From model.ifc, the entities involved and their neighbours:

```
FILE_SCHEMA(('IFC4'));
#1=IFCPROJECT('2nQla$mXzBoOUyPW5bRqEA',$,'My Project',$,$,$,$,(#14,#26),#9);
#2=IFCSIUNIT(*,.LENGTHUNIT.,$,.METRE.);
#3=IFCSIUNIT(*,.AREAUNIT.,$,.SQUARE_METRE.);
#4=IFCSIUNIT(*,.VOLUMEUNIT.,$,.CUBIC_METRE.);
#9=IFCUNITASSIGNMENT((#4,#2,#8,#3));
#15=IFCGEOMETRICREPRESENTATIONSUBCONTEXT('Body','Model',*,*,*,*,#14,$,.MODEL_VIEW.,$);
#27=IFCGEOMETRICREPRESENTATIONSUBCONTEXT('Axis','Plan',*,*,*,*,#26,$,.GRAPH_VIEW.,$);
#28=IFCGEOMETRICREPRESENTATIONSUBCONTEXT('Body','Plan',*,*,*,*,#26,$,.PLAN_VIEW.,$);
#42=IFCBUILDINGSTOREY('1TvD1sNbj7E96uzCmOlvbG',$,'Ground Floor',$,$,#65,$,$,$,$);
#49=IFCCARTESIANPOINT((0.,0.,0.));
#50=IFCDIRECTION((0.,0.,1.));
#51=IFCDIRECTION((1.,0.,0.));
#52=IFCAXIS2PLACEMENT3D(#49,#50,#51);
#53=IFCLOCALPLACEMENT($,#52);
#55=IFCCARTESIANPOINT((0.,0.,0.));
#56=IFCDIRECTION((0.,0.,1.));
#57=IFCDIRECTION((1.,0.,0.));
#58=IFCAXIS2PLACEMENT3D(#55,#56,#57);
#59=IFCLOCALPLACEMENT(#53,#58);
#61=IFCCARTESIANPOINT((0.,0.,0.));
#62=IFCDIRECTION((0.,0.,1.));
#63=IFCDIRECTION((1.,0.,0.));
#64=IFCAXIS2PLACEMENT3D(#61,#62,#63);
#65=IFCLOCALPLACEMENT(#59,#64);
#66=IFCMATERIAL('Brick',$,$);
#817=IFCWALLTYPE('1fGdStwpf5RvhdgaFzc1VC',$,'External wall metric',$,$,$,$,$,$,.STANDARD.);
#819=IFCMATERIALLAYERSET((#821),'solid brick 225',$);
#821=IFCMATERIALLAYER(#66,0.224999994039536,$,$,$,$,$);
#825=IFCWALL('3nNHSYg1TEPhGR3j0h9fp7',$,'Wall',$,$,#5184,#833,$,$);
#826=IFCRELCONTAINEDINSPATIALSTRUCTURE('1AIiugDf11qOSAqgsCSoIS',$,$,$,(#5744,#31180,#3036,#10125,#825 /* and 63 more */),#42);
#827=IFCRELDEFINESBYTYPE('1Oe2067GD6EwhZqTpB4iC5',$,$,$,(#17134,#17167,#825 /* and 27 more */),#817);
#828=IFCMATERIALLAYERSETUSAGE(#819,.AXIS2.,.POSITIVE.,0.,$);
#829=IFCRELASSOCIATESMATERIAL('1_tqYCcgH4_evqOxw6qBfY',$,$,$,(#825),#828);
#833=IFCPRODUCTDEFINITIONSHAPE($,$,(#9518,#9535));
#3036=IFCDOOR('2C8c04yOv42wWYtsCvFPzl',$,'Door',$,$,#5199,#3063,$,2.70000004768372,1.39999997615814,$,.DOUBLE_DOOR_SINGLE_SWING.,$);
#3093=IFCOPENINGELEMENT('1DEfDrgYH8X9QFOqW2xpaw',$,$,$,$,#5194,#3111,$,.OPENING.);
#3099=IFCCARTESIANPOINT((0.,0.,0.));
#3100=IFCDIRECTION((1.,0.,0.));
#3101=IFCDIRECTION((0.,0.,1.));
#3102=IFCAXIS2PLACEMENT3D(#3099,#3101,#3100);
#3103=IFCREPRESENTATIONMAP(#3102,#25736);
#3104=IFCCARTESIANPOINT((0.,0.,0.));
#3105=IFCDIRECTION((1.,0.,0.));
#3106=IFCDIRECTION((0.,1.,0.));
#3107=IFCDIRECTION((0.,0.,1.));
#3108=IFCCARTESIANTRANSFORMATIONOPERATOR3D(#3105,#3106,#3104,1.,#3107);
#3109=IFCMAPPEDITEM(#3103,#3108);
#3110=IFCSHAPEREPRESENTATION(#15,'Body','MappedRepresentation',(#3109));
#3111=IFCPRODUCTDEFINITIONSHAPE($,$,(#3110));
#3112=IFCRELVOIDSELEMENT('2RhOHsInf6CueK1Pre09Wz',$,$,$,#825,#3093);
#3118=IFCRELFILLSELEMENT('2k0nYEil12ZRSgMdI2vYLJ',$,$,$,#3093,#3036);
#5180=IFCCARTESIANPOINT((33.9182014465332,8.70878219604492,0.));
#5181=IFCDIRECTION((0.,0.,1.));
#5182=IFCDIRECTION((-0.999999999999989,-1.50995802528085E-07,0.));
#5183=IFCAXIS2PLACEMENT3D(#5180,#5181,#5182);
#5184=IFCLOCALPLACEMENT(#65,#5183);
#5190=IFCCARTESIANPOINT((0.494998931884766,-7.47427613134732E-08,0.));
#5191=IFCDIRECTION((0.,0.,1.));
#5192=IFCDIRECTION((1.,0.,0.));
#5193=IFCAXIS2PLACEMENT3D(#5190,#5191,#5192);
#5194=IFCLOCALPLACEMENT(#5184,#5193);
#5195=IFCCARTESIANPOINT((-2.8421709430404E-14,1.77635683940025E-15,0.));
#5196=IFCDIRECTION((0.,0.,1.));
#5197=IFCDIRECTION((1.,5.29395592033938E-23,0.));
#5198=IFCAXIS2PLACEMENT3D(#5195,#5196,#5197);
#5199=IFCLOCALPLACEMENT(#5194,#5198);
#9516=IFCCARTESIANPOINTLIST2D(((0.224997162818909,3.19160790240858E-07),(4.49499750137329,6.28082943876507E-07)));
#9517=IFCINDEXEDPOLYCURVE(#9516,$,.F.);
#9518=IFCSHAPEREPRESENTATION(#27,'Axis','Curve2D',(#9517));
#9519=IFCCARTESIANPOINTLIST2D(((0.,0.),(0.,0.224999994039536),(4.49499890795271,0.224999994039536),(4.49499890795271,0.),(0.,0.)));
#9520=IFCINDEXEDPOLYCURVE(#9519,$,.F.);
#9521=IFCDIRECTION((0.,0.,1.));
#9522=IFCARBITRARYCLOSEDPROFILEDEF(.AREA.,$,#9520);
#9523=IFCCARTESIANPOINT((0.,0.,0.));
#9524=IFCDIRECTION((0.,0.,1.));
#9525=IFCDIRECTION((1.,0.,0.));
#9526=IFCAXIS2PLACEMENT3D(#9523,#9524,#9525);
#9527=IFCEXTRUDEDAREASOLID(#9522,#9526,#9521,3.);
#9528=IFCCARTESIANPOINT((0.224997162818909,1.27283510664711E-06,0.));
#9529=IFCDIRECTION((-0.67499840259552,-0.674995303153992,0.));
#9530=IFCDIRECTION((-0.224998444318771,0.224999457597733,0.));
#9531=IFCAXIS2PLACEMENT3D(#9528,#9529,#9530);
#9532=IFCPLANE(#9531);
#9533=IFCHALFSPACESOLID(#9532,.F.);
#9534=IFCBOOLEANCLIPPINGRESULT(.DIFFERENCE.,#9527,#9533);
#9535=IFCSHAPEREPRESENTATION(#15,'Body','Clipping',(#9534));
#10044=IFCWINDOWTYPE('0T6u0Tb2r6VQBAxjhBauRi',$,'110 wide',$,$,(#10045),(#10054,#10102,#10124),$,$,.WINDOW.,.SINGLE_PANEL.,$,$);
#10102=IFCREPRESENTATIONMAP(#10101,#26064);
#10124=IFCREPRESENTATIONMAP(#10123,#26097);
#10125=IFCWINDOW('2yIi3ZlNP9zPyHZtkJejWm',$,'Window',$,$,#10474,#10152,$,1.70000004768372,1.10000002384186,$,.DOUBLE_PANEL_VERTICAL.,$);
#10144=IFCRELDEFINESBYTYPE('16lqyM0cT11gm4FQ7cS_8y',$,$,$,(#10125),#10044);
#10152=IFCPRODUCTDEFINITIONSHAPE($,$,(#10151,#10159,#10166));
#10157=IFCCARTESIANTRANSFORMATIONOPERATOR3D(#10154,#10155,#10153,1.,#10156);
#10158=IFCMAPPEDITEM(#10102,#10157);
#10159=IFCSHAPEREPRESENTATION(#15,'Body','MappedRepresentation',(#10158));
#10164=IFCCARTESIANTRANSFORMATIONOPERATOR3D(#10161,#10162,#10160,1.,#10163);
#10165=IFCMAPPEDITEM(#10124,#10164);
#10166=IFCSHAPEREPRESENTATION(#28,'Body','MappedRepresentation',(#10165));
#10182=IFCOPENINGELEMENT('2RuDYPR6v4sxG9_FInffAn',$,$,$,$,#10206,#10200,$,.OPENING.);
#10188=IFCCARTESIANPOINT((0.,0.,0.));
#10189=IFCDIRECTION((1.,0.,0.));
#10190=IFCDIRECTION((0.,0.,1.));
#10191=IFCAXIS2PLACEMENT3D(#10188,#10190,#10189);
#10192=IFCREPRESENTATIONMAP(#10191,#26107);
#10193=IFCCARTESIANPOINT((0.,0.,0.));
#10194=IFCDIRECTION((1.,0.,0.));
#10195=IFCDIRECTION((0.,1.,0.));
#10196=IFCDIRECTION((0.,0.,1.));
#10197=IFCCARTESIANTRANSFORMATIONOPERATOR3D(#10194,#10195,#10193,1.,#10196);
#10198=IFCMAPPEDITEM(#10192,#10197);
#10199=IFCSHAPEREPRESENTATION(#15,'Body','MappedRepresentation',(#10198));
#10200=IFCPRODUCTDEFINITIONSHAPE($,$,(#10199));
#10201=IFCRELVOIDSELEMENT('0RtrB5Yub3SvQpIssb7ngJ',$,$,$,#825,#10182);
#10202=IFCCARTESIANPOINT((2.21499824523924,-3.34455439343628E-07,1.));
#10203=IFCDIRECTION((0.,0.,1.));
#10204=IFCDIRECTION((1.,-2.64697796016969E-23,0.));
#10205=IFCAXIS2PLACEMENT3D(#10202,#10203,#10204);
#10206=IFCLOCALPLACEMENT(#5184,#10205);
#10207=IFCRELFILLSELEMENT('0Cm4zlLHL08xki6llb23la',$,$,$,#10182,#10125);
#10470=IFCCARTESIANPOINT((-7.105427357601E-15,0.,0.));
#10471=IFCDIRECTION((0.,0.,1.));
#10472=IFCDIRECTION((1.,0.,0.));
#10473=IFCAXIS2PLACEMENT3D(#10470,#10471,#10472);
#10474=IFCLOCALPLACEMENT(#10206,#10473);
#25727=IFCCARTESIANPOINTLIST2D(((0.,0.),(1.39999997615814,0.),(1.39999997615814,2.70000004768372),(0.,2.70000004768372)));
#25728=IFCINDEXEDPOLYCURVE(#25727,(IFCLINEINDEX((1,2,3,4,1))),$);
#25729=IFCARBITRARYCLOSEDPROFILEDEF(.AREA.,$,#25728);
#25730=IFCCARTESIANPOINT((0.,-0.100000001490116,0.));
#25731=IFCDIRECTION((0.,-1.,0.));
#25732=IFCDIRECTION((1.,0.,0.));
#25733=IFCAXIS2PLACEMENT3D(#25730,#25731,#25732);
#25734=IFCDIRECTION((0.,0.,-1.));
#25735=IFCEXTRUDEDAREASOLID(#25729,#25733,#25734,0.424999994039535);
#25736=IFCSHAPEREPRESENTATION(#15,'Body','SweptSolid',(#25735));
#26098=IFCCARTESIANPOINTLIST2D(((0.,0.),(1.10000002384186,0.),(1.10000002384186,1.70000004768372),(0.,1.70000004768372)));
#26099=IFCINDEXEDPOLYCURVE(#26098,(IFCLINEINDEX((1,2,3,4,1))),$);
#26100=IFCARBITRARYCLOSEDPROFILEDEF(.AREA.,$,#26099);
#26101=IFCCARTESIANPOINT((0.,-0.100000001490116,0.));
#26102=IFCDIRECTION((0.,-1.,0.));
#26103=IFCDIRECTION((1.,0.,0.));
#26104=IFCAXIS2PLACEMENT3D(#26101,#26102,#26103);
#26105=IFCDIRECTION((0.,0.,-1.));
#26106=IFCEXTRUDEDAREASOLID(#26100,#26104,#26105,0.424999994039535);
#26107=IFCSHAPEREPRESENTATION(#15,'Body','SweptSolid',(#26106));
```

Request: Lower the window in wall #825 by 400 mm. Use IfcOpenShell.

```python
import numpy as np
import ifcopenshell
import ifcopenshell.api.geometry
import ifcopenshell.util.placement
import ifcopenshell.util.unit

model = ifcopenshell.open("model.ifc")
unit_scale = ifcopenshell.util.unit.calculate_unit_scale(model)

window = model.by_id(10125)
opening = window.FillsVoids[0].RelatingOpeningElement
dz = -0.4 / unit_scale

shift = np.array([0.0, 0.0, dz])
# The window is placed relative to its opening, so it follows when the opening moves.
matrix = ifcopenshell.util.placement.get_local_placement(opening.ObjectPlacement)
matrix[:3, 3] += shift
ifcopenshell.api.geometry.edit_object_placement(
    model, product=opening, matrix=matrix, is_si=False, should_transform_children=True
)

print(f"moved by {dz * unit_scale:+.3f} m")

model.write("model_rev.ifc")
```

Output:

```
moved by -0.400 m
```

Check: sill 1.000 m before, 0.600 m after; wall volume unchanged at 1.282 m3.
